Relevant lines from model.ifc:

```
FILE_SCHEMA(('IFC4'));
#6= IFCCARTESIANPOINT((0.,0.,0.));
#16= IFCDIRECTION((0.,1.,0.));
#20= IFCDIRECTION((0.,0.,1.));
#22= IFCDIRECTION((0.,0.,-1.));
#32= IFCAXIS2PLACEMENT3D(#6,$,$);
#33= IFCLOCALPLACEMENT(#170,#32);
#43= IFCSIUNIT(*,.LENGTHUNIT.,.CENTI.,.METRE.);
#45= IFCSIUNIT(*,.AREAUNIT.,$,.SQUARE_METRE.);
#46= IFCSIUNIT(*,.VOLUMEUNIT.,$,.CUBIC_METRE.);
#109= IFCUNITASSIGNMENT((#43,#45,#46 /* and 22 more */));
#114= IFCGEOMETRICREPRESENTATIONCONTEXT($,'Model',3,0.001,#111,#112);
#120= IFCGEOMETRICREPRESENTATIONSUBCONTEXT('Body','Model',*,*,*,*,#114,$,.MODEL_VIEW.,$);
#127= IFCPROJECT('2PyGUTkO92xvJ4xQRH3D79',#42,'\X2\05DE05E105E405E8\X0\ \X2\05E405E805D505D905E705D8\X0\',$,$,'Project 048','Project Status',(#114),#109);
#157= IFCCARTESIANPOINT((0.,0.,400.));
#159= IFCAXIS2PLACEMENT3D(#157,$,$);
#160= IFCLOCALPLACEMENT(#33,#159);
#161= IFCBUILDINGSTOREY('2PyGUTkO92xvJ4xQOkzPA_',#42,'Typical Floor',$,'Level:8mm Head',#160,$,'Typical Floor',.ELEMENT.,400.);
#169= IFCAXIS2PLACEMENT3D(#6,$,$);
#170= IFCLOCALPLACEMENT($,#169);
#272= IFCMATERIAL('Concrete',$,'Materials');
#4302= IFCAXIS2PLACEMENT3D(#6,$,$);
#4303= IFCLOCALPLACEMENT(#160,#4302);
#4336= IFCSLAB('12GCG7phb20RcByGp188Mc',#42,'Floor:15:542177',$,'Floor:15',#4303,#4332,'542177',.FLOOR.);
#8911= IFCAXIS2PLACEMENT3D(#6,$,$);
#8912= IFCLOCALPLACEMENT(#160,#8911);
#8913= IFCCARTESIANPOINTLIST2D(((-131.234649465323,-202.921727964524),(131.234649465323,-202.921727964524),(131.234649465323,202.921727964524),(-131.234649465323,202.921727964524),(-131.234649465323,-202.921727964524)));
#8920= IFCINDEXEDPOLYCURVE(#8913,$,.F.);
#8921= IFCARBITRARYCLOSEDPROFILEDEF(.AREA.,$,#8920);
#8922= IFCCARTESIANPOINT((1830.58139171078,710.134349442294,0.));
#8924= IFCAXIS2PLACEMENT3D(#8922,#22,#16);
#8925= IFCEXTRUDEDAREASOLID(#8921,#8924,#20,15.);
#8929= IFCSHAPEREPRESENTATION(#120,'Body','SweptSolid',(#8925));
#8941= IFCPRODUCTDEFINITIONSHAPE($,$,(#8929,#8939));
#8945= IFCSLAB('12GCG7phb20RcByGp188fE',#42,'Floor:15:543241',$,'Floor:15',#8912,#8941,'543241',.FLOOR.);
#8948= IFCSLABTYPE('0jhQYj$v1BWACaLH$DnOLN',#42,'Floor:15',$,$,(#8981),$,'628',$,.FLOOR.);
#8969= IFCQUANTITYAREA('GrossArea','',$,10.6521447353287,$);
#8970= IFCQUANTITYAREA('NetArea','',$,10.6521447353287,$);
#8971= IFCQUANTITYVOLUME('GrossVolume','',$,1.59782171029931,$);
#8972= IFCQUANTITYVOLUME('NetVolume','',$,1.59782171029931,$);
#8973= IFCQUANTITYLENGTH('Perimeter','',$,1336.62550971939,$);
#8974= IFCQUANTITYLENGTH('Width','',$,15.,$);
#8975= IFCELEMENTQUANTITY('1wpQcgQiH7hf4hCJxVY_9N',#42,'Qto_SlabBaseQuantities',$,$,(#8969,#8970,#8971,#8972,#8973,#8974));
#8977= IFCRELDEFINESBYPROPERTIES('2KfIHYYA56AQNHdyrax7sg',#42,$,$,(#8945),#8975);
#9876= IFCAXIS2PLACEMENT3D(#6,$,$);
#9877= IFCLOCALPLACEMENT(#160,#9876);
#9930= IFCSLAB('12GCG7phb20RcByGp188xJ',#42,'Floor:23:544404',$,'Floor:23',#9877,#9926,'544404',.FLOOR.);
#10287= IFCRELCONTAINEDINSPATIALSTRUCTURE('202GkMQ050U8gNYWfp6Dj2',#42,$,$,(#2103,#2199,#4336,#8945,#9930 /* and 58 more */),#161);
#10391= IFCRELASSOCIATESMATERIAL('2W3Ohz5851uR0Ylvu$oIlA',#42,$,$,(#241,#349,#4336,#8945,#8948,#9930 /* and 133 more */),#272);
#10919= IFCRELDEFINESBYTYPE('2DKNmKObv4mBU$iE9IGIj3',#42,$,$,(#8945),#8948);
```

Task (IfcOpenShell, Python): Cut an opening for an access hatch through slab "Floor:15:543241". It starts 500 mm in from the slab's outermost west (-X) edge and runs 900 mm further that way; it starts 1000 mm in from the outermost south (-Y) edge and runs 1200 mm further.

```python
import numpy as np
import ifcopenshell
import ifcopenshell.api.feature
import ifcopenshell.api.geometry
import ifcopenshell.api.pset
import ifcopenshell.api.root
import ifcopenshell.geom
import ifcopenshell.util.element
import ifcopenshell.util.placement
import ifcopenshell.util.representation
import ifcopenshell.util.shape
import ifcopenshell.util.unit

model = ifcopenshell.open("model.ifc")
unit_scale = ifcopenshell.util.unit.calculate_unit_scale(model)
area_scale = ifcopenshell.util.unit.calculate_unit_scale(model, "AREAUNIT")
volume_scale = ifcopenshell.util.unit.calculate_unit_scale(model, "VOLUMEUNIT")
settings = ifcopenshell.geom.settings()


def volume(element):
    """Net volume in cubic metres, openings subtracted."""
    shape = ifcopenshell.geom.create_shape(settings, element)
    return ifcopenshell.util.shape.get_volume(shape.geometry)


slab = model.by_id(8945)
before = volume(slab)

# Extent in the slab's own axes, in metres. The edges named are its -X and -Y sides.
slab_shape = ifcopenshell.geom.create_shape(settings, slab)
vertices = ifcopenshell.util.shape.get_vertices(slab_shape.geometry)
x_min, y_min, bottom = vertices.min(axis=0)
top = vertices[:, 2].max()

opening = ifcopenshell.api.root.create_entity(model, ifc_class="IfcOpeningElement", name="Access hatch opening", predefined_type="OPENING")
context = ifcopenshell.util.representation.get_context(model, "Model", "Body", "MODEL_VIEW")
width, depth = 0.9, 1.2
outline = [(0.0, 0.0), (width, 0.0), (width, depth), (0.0, depth), (0.0, 0.0)]
# Overshoot both faces by 50 mm so the cut is clean.
shape = ifcopenshell.api.geometry.add_slab_representation(
    model, context=context, depth=top - bottom + 0.1, polyline=outline
)
ifcopenshell.api.geometry.assign_representation(model, product=opening, representation=shape)

matrix = ifcopenshell.util.placement.get_local_placement(slab.ObjectPlacement)
matrix[:, 3] = matrix @ np.append(np.array([x_min + 0.5, y_min + 1, bottom - 0.05]) / unit_scale, 1.0)
ifcopenshell.api.geometry.edit_object_placement(model, product=opening, matrix=matrix, is_si=False)
ifcopenshell.api.feature.add_feature(model, feature=opening, element=slab)

after = volume(slab)

# Update the slab's stored quantities.
qto = model.by_id(ifcopenshell.util.element.get_pset(slab, "Qto_SlabBaseQuantities", should_inherit=False)["id"])
ifcopenshell.api.pset.edit_qto(model, qto=qto, properties={
    "NetArea": after / (top - bottom) / area_scale,
    "NetVolume": after / volume_scale,
})

print(f"slab volume {before:.3f} -> {after:.3f} m3")

model.write("model_updated.ifc")
```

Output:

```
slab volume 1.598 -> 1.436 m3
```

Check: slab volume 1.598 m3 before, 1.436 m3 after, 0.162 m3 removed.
